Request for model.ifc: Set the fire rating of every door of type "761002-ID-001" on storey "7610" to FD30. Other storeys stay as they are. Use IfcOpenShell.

First a look at what the model holds.

```python
import ifcopenshell
import ifcopenshell.util.element

model = ifcopenshell.open("model.ifc")
print(model.schema)
storey = next(s for s in model.by_type("IfcBuildingStorey") if s.Name == "7610")
doors = [e for e in ifcopenshell.util.element.get_decomposition(storey) if e.is_a("IfcDoor")]
seen = {}
for e in doors:
    element_type = ifcopenshell.util.element.get_type(e)
    key = (element_type.Name if element_type != e and element_type else None, ifcopenshell.util.element.get_pset(e, "Pset_DoorCommon", "FireRating"))
    seen[key] = seen.get(key, 0) + 1
for (name, value), count in sorted(seen.items(), key=str):
    print(count, "x", name, "|", value)
```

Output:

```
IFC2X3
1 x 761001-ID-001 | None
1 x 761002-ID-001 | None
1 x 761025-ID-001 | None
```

```python
import ifcopenshell
import ifcopenshell.api.pset
import ifcopenshell.util.element

model = ifcopenshell.open("model.ifc")

storey = next(s for s in model.by_type("IfcBuildingStorey") if s.Name == "7610")
doors = [e for e in ifcopenshell.util.element.get_decomposition(storey) if e.is_a("IfcDoor")]

count = 0
for e in doors:
    element_type = ifcopenshell.util.element.get_type(e)
    if element_type in (None, e) or element_type.Name != "761002-ID-001":
        continue
    # add_pset returns the element's existing set when there is one.
    pset = ifcopenshell.api.pset.add_pset(model, product=e, name="Pset_DoorCommon")
    ifcopenshell.api.pset.edit_pset(model, pset=pset, properties={"FireRating": "FD30"})
    count += 1

print(count, "doors updated")

model.write("model_v2.ifc")
```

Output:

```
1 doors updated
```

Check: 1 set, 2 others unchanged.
